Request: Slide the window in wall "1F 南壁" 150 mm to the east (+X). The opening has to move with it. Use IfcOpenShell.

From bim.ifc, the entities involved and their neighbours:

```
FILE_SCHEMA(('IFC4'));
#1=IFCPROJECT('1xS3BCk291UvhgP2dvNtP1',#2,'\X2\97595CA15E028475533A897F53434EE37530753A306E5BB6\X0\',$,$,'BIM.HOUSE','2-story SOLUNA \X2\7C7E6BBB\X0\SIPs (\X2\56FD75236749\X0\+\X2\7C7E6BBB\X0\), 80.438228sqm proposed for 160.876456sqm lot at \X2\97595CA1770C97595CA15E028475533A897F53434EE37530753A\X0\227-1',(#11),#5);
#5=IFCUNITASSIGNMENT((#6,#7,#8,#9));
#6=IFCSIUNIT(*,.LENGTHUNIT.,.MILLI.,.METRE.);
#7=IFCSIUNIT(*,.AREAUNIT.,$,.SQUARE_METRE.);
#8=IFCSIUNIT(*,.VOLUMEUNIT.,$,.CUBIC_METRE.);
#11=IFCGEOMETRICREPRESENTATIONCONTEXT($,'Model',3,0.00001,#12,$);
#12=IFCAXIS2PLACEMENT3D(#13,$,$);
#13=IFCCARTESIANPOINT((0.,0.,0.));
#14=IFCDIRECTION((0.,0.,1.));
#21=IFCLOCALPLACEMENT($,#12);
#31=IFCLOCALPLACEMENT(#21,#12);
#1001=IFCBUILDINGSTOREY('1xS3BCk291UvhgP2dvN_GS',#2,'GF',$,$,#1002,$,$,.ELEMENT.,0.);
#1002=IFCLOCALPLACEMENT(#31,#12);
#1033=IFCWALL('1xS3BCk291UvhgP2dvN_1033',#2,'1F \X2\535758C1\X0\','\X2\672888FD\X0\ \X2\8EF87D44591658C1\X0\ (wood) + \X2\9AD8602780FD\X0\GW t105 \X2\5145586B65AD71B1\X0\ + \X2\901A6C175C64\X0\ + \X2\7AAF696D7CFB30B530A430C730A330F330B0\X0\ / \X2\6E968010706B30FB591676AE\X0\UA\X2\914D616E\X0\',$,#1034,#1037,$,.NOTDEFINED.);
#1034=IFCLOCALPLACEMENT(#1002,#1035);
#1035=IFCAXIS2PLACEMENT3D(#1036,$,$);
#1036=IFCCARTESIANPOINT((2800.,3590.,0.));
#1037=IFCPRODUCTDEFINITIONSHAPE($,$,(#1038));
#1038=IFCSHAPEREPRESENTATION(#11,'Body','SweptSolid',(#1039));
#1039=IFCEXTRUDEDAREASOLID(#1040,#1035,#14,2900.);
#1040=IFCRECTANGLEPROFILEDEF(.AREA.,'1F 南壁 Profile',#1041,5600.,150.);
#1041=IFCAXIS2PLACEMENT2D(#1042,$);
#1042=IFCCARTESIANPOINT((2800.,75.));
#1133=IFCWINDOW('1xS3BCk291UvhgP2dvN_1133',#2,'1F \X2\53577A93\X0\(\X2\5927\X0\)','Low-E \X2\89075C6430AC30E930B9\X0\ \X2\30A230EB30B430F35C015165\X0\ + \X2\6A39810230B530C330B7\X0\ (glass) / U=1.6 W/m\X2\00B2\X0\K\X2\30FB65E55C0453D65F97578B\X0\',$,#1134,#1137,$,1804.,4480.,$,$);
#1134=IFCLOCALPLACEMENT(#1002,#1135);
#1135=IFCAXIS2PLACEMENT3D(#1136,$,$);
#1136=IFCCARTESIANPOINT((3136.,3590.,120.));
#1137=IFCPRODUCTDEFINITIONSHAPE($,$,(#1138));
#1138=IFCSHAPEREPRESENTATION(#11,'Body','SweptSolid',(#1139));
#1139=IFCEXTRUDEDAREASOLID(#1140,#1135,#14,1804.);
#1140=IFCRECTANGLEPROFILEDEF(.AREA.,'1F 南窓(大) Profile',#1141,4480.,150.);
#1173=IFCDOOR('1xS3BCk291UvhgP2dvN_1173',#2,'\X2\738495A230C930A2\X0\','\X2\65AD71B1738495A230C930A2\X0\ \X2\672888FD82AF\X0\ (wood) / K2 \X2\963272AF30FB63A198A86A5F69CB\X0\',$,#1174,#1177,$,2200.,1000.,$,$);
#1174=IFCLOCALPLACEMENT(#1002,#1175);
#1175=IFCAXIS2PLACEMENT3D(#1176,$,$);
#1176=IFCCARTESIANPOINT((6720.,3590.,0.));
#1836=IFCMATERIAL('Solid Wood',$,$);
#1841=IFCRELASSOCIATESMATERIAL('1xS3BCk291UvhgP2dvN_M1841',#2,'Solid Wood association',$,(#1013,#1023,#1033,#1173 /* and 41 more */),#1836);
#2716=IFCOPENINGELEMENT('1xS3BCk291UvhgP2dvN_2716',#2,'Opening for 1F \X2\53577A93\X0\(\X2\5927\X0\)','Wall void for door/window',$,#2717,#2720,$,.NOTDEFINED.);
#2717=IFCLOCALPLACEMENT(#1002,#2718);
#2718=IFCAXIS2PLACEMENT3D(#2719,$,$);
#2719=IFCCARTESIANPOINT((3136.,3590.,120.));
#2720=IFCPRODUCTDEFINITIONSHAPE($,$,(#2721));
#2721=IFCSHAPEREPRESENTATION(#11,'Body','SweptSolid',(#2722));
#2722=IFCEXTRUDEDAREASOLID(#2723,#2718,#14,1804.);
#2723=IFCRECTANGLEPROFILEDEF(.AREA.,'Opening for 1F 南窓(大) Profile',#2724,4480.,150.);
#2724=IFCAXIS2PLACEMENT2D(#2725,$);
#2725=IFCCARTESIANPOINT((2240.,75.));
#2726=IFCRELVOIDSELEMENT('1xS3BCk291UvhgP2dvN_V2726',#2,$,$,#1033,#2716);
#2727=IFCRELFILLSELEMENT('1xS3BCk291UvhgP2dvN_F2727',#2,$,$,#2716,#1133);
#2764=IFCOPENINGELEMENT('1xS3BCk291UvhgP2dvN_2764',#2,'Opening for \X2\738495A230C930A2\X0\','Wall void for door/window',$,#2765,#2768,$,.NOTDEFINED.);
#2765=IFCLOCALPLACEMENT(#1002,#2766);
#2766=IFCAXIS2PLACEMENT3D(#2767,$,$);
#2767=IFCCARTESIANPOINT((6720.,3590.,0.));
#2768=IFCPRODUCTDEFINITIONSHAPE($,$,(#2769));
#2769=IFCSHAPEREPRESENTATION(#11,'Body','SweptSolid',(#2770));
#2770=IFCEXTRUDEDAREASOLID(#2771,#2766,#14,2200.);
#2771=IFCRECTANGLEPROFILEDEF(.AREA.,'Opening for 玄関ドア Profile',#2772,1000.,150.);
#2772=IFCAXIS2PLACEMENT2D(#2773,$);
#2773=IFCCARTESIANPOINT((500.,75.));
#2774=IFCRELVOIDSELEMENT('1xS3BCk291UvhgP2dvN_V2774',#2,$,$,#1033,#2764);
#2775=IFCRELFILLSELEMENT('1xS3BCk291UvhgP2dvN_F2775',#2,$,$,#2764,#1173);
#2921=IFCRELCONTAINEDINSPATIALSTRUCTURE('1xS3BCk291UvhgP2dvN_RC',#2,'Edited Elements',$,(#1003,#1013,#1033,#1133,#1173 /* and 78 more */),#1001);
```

```python
import ifcopenshell
import ifcopenshell.api.geometry
import ifcopenshell.util.placement

model = ifcopenshell.open("bim.ifc")

window = model.by_guid("1xS3BCk291UvhgP2dvN_1133")
opening = window.FillsVoids[0].RelatingOpeningElement
wall = opening.VoidsElements[0].RelatingBuildingElement

wall_matrix = ifcopenshell.util.placement.get_local_placement(wall.ObjectPlacement)
shift = wall_matrix[:3, 0] * 150.0
before = ifcopenshell.util.placement.get_local_placement(window.ObjectPlacement)[:3, 3].copy()

# The window is not placed relative to its opening, so move both.
for product in (opening, window):
    matrix = ifcopenshell.util.placement.get_local_placement(product.ObjectPlacement)
    matrix[:3, 3] += shift
    ifcopenshell.api.geometry.edit_object_placement(model, product=product, matrix=matrix, is_si=False)

after = ifcopenshell.util.placement.get_local_placement(window.ObjectPlacement)[:3, 3]
print("window moved by", (after - before).round(3) + 0.0)

model.write("bim_v2.ifc")
```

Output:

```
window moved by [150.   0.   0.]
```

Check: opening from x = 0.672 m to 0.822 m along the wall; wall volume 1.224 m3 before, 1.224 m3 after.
